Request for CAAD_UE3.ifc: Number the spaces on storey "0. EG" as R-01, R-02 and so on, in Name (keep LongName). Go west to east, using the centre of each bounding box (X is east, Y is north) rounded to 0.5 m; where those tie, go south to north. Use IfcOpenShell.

First a look at what the model holds.

```python
import ifcopenshell
import ifcopenshell.util.element
import ifcopenshell.util.placement

model = ifcopenshell.open("CAAD_UE3.ifc")
print(model.schema)
storey = next(s for s in model.by_type("IfcBuildingStorey") if s.Name == "0. EG")
spaces = [e for e in ifcopenshell.util.element.get_decomposition(storey) if e.is_a("IfcSpace")]
for e in sorted(spaces, key=lambda e: e.id()):
    origin = ifcopenshell.util.placement.get_local_placement(e.ObjectPlacement)[:3, 3]
    print(e.id(), e.Name, e.LongName, origin.round(2) + 0.0, sep=" | ")
```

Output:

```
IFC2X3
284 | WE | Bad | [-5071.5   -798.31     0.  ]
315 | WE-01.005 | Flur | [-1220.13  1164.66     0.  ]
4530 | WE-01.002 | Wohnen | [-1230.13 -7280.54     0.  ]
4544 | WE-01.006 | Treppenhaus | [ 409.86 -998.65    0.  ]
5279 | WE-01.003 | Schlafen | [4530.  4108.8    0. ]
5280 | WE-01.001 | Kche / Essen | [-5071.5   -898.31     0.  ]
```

```python
import ifcopenshell
import ifcopenshell.geom
import ifcopenshell.util.element
import ifcopenshell.util.shape

model = ifcopenshell.open("CAAD_UE3.ifc")
settings = ifcopenshell.geom.settings()
settings.set("use-world-coords", True)


def centre(element):
    shape = ifcopenshell.geom.create_shape(settings, element)
    return ifcopenshell.util.shape.get_bbox_centroid(shape.geometry)


storey = next(s for s in model.by_type("IfcBuildingStorey") if s.Name == "0. EG")
spaces = [e for e in ifcopenshell.util.element.get_decomposition(storey) if e.is_a("IfcSpace")]

# Insertion points can sit at a corner or the storey origin, so sort by the geometry (in metres).
centres = {e: centre(e) for e in spaces}
spaces.sort(key=lambda e: (round(centres[e][0] / 0.5), centres[e][1]))

for i, e in enumerate(spaces, start=1):
    number = f"R-{i:02d}"
    e.Name = number
    print(e.id(), number)

model.write("CAAD_UE3_rev.ifc")
```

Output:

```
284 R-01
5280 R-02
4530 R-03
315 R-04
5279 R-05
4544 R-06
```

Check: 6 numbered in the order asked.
